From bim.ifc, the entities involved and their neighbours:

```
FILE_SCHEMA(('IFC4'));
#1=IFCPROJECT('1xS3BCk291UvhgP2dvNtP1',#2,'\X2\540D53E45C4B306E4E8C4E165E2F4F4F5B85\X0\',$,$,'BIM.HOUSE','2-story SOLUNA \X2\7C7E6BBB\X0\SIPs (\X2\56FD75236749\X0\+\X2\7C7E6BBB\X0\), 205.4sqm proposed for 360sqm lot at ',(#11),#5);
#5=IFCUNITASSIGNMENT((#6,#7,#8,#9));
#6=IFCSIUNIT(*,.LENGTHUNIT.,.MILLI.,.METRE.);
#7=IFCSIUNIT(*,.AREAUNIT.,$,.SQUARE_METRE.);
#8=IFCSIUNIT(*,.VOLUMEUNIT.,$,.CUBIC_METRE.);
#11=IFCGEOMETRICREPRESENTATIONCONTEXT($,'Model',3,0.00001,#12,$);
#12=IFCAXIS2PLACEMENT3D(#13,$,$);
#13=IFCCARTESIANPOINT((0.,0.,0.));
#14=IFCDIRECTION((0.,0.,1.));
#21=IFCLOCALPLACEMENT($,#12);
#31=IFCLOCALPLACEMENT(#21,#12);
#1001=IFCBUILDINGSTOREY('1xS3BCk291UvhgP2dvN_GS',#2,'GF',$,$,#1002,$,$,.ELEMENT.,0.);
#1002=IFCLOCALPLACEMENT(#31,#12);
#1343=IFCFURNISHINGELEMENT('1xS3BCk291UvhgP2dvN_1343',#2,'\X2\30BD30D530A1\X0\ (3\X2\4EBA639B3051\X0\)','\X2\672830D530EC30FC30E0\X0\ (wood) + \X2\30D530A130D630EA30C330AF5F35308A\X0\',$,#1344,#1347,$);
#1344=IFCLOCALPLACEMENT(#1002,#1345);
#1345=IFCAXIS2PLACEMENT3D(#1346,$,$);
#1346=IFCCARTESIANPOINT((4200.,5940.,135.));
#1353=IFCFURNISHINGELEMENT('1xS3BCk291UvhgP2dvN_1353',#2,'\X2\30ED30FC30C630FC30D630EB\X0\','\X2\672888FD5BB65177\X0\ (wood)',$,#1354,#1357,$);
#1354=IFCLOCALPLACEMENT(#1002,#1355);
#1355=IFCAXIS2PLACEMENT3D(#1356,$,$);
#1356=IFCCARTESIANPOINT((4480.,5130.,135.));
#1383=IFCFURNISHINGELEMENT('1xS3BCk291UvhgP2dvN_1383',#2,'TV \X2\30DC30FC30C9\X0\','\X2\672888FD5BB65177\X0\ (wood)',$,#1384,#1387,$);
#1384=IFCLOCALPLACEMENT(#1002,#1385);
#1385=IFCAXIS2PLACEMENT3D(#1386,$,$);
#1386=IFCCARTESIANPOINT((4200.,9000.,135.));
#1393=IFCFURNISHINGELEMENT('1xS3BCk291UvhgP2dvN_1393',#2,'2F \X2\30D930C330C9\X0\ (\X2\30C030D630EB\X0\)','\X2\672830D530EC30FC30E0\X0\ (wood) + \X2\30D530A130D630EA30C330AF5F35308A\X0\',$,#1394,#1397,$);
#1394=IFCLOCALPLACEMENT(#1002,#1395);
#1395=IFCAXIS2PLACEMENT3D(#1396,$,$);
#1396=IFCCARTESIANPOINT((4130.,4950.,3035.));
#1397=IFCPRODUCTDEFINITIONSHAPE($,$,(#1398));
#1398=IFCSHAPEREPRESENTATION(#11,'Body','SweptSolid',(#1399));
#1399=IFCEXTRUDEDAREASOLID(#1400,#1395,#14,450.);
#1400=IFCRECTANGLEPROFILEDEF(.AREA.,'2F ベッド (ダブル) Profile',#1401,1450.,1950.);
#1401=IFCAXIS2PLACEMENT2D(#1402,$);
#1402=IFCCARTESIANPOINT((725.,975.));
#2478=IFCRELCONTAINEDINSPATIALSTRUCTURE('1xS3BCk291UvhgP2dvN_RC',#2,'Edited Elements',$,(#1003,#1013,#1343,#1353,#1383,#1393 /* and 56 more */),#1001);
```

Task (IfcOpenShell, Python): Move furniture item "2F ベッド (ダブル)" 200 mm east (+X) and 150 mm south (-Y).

```python
import ifcopenshell
import ifcopenshell.api.geometry
import ifcopenshell.util.placement
import ifcopenshell.util.unit

model = ifcopenshell.open("bim.ifc")
unit_scale = ifcopenshell.util.unit.calculate_unit_scale(model)

item = model.by_id(1393)
matrix = ifcopenshell.util.placement.get_local_placement(item.ObjectPlacement)
matrix[0, 3] += 0.2 / unit_scale
matrix[1, 3] -= 0.15 / unit_scale
ifcopenshell.api.geometry.edit_object_placement(model, product=item, matrix=matrix, is_si=False)

print(ifcopenshell.util.placement.get_local_placement(item.ObjectPlacement).round(3) + 0.0)

model.write("bim_updated.ifc")
```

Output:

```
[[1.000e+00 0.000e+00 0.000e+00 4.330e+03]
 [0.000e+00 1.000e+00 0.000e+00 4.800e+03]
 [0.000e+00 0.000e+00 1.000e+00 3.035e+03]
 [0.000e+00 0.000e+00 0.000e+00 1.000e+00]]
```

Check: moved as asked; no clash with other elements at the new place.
